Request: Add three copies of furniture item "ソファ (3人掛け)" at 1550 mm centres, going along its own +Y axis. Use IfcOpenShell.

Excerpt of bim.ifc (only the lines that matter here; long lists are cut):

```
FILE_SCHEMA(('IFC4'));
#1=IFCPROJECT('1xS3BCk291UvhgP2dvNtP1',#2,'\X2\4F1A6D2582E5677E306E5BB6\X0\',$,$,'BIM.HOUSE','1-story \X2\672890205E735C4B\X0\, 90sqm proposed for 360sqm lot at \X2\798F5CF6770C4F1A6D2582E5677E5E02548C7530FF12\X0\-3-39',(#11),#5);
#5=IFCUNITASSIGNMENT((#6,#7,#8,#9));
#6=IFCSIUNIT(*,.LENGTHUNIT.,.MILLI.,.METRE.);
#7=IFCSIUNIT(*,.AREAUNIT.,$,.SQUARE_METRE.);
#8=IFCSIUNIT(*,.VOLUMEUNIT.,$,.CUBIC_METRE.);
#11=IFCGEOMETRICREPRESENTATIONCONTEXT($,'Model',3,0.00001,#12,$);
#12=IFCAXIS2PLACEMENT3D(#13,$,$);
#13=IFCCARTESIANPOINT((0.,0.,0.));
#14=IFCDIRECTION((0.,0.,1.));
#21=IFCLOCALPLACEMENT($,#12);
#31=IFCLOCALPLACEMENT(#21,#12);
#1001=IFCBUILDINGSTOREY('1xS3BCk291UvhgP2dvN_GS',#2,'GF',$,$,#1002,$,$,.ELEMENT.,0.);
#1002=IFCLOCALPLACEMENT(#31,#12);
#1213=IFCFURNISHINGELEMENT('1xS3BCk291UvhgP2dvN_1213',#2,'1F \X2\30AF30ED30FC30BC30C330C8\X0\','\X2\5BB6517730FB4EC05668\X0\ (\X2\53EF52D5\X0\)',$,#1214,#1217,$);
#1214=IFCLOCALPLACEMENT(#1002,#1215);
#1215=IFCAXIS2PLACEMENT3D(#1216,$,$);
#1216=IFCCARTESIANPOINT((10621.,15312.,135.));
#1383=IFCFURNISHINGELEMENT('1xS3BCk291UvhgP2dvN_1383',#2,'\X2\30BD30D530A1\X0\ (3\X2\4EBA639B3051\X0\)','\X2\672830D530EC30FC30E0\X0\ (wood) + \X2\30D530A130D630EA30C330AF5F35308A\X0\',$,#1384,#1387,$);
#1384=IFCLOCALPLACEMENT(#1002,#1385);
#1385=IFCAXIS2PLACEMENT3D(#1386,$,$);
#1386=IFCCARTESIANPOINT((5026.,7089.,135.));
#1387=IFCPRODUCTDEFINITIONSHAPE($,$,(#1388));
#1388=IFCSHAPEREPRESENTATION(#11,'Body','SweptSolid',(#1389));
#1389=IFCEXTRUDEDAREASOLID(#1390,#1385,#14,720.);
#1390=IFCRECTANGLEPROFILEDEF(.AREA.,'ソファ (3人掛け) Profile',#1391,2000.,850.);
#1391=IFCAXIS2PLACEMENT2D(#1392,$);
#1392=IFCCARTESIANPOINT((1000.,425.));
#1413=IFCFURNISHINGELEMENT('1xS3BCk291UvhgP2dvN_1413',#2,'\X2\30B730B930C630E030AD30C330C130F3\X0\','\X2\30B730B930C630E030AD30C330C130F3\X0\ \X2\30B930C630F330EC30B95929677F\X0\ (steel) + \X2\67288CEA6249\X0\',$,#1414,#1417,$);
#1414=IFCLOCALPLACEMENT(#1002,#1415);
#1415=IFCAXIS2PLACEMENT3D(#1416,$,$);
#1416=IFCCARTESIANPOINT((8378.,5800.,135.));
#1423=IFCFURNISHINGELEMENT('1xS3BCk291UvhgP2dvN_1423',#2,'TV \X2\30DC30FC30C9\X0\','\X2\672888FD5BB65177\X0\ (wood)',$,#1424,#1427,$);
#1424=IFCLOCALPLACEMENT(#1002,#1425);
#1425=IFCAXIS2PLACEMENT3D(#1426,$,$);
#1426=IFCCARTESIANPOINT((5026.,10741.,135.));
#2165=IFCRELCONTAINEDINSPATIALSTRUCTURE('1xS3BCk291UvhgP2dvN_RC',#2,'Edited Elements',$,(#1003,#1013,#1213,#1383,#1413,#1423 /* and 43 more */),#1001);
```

```python
import ifcopenshell
import ifcopenshell.api.geometry
import ifcopenshell.api.root
import ifcopenshell.util.element
import ifcopenshell.util.placement
import ifcopenshell.util.unit

model = ifcopenshell.open("bim.ifc")
unit_scale = ifcopenshell.util.unit.calculate_unit_scale(model)


def reuse_history(source, copy):
    """copy_class also copies each property set's owner history, people and application; keep the originals."""
    for rel in copy.IsDefinedBy:
        if rel.is_a("IfcRelDefinesByProperties") and (history := rel.RelatingPropertyDefinition.OwnerHistory):
            rel.RelatingPropertyDefinition.OwnerHistory = source.OwnerHistory
            ifcopenshell.util.element.remove_deep2(model, history)


source = model.by_guid("1xS3BCk291UvhgP2dvN_1383")
base = ifcopenshell.util.placement.get_local_placement(source.ObjectPlacement)
step = base[:3, 1] * 1.55 / unit_scale

for i in range(1, 4):
    copy = ifcopenshell.api.root.copy_class(model, product=source)
    copy.Representation = ifcopenshell.util.element.copy_deep(
        model, source.Representation, exclude=["IfcGeometricRepresentationContext", "IfcRepresentationMap"]
    )
    reuse_history(source, copy)
    matrix = base.copy()
    matrix[:3, 3] += i * step
    print("added at", matrix[:3, 3].round(3) + 0.0)
    ifcopenshell.api.geometry.edit_object_placement(model, product=copy, matrix=matrix, is_si=False)

model.write("bim_updated.ifc")
```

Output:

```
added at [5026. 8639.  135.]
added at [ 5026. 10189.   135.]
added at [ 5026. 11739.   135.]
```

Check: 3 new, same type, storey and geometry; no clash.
